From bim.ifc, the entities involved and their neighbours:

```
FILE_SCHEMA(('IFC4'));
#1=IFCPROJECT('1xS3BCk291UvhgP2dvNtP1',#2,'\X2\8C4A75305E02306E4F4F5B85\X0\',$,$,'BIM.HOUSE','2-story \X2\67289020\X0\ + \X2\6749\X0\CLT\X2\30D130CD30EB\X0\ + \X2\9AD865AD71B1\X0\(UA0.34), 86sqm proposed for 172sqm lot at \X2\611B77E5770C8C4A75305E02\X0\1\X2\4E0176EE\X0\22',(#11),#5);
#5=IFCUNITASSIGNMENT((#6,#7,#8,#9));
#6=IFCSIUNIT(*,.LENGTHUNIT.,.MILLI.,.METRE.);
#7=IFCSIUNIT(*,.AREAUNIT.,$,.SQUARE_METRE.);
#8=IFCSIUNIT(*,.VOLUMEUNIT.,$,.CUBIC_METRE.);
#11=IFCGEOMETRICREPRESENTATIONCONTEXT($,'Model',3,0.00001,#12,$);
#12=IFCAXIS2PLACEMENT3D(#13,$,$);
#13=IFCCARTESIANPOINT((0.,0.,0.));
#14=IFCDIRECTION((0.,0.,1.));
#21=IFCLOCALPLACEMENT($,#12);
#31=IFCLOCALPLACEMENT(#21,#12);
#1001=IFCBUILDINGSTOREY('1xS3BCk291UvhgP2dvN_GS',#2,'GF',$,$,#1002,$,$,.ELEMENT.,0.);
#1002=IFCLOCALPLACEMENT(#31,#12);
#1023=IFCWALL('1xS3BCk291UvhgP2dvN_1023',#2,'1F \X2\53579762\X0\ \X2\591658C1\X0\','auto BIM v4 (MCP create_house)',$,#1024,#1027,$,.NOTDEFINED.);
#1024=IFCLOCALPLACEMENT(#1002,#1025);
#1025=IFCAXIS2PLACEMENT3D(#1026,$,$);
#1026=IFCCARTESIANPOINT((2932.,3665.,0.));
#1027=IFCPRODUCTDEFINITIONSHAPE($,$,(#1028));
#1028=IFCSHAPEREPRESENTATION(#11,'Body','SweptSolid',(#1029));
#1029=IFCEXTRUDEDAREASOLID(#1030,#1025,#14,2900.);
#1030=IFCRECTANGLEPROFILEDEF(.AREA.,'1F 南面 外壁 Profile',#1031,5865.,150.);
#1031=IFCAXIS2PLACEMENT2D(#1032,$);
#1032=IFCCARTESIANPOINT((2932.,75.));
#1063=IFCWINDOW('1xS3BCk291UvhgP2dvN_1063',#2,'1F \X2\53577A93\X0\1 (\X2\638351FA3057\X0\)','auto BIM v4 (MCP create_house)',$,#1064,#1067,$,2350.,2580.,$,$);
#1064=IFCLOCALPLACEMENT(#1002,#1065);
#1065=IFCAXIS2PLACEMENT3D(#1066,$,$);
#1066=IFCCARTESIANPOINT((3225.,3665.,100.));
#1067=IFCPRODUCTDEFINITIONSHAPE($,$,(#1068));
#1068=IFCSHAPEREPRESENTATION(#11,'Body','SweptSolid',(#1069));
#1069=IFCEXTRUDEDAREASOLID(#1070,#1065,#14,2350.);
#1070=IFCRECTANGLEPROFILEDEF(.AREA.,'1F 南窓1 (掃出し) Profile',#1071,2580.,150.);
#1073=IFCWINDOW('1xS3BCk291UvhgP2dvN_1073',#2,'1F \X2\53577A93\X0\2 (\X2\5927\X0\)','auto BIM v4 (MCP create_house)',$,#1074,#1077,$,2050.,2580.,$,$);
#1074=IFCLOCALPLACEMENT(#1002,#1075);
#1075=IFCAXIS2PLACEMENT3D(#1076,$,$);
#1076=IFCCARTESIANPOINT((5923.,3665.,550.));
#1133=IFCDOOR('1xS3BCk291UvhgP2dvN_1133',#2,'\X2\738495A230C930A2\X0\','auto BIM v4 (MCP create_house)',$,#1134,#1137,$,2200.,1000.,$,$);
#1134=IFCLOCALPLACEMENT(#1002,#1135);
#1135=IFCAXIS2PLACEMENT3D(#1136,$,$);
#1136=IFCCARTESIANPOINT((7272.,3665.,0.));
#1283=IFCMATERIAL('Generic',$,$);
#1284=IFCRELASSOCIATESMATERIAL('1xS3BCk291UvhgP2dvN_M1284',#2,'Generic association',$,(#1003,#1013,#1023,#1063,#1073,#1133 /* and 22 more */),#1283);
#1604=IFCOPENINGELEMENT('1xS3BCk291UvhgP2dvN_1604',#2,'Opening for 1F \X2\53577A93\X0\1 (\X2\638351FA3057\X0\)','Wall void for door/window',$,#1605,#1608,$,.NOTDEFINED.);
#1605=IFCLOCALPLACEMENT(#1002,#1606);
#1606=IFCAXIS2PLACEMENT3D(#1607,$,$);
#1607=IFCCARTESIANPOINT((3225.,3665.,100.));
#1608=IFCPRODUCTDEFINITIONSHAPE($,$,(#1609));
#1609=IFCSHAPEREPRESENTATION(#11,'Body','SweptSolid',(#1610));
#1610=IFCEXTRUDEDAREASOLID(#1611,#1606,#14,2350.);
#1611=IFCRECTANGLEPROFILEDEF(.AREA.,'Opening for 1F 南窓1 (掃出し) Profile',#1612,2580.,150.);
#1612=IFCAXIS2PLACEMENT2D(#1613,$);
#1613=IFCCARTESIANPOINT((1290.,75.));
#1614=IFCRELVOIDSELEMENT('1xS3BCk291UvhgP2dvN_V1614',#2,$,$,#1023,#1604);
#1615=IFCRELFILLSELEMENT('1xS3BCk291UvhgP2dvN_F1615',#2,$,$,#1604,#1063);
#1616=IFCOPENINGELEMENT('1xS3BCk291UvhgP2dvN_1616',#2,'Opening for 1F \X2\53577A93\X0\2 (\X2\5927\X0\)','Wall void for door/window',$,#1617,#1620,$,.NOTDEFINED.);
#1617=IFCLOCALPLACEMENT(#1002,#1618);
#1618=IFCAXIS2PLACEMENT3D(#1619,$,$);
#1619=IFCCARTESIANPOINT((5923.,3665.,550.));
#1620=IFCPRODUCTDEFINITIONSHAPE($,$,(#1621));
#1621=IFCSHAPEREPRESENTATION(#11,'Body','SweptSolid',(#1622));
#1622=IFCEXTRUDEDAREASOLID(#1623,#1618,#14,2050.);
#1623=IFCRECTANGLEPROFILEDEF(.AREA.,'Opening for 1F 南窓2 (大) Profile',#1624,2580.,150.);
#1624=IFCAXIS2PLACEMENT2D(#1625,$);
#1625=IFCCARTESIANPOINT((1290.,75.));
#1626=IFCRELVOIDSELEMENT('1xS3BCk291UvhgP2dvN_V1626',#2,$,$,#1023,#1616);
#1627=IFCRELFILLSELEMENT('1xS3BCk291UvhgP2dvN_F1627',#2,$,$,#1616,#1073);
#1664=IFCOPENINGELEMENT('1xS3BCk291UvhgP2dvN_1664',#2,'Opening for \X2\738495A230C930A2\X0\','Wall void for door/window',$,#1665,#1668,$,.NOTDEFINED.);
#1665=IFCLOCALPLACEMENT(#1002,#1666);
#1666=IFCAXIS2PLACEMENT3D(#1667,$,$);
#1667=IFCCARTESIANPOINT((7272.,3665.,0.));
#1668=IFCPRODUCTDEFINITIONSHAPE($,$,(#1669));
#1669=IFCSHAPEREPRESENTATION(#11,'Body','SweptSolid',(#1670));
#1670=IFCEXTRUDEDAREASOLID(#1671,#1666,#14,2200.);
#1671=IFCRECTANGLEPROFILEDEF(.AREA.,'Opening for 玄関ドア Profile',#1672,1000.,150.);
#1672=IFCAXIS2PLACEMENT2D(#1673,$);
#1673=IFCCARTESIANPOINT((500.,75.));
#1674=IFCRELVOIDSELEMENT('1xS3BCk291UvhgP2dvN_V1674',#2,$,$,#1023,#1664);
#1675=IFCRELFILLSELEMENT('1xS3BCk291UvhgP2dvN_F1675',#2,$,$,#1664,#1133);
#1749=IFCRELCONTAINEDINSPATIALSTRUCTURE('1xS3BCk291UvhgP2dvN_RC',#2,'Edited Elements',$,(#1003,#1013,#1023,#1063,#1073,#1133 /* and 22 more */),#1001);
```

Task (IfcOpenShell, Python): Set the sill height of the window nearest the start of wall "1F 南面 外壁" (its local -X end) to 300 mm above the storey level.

```python
import numpy as np
import ifcopenshell
import ifcopenshell.api.geometry
import ifcopenshell.geom
import ifcopenshell.util.element
import ifcopenshell.util.placement
import ifcopenshell.util.shape
import ifcopenshell.util.unit

model = ifcopenshell.open("bim.ifc")
unit_scale = ifcopenshell.util.unit.calculate_unit_scale(model)

window = model.by_guid("1xS3BCk291UvhgP2dvN_1063")
opening = window.FillsVoids[0].RelatingOpeningElement
storey = ifcopenshell.util.element.get_container(window, ifc_class="IfcBuildingStorey")
level = ifcopenshell.util.placement.get_local_placement(storey.ObjectPlacement)[2, 3]

# The opening's origin need not be at the sill, so measure its lowest point.
shape = ifcopenshell.geom.create_shape(ifcopenshell.geom.settings(), opening)
bottom = ifcopenshell.util.shape.get_shape_bottom_elevation(shape, shape.geometry) / unit_scale
dz = level + 0.3 / unit_scale - bottom

shift = np.array([0.0, 0.0, dz])
# The window is not placed relative to its opening, so move both.
for product in (opening, window):
    matrix = ifcopenshell.util.placement.get_local_placement(product.ObjectPlacement)
    matrix[:3, 3] += shift
    ifcopenshell.api.geometry.edit_object_placement(model, product=product, matrix=matrix, is_si=False)

print(f"moved by {dz * unit_scale:+.3f} m")

model.write("bim-out.ifc")
```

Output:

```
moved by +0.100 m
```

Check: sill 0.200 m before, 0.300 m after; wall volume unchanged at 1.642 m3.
